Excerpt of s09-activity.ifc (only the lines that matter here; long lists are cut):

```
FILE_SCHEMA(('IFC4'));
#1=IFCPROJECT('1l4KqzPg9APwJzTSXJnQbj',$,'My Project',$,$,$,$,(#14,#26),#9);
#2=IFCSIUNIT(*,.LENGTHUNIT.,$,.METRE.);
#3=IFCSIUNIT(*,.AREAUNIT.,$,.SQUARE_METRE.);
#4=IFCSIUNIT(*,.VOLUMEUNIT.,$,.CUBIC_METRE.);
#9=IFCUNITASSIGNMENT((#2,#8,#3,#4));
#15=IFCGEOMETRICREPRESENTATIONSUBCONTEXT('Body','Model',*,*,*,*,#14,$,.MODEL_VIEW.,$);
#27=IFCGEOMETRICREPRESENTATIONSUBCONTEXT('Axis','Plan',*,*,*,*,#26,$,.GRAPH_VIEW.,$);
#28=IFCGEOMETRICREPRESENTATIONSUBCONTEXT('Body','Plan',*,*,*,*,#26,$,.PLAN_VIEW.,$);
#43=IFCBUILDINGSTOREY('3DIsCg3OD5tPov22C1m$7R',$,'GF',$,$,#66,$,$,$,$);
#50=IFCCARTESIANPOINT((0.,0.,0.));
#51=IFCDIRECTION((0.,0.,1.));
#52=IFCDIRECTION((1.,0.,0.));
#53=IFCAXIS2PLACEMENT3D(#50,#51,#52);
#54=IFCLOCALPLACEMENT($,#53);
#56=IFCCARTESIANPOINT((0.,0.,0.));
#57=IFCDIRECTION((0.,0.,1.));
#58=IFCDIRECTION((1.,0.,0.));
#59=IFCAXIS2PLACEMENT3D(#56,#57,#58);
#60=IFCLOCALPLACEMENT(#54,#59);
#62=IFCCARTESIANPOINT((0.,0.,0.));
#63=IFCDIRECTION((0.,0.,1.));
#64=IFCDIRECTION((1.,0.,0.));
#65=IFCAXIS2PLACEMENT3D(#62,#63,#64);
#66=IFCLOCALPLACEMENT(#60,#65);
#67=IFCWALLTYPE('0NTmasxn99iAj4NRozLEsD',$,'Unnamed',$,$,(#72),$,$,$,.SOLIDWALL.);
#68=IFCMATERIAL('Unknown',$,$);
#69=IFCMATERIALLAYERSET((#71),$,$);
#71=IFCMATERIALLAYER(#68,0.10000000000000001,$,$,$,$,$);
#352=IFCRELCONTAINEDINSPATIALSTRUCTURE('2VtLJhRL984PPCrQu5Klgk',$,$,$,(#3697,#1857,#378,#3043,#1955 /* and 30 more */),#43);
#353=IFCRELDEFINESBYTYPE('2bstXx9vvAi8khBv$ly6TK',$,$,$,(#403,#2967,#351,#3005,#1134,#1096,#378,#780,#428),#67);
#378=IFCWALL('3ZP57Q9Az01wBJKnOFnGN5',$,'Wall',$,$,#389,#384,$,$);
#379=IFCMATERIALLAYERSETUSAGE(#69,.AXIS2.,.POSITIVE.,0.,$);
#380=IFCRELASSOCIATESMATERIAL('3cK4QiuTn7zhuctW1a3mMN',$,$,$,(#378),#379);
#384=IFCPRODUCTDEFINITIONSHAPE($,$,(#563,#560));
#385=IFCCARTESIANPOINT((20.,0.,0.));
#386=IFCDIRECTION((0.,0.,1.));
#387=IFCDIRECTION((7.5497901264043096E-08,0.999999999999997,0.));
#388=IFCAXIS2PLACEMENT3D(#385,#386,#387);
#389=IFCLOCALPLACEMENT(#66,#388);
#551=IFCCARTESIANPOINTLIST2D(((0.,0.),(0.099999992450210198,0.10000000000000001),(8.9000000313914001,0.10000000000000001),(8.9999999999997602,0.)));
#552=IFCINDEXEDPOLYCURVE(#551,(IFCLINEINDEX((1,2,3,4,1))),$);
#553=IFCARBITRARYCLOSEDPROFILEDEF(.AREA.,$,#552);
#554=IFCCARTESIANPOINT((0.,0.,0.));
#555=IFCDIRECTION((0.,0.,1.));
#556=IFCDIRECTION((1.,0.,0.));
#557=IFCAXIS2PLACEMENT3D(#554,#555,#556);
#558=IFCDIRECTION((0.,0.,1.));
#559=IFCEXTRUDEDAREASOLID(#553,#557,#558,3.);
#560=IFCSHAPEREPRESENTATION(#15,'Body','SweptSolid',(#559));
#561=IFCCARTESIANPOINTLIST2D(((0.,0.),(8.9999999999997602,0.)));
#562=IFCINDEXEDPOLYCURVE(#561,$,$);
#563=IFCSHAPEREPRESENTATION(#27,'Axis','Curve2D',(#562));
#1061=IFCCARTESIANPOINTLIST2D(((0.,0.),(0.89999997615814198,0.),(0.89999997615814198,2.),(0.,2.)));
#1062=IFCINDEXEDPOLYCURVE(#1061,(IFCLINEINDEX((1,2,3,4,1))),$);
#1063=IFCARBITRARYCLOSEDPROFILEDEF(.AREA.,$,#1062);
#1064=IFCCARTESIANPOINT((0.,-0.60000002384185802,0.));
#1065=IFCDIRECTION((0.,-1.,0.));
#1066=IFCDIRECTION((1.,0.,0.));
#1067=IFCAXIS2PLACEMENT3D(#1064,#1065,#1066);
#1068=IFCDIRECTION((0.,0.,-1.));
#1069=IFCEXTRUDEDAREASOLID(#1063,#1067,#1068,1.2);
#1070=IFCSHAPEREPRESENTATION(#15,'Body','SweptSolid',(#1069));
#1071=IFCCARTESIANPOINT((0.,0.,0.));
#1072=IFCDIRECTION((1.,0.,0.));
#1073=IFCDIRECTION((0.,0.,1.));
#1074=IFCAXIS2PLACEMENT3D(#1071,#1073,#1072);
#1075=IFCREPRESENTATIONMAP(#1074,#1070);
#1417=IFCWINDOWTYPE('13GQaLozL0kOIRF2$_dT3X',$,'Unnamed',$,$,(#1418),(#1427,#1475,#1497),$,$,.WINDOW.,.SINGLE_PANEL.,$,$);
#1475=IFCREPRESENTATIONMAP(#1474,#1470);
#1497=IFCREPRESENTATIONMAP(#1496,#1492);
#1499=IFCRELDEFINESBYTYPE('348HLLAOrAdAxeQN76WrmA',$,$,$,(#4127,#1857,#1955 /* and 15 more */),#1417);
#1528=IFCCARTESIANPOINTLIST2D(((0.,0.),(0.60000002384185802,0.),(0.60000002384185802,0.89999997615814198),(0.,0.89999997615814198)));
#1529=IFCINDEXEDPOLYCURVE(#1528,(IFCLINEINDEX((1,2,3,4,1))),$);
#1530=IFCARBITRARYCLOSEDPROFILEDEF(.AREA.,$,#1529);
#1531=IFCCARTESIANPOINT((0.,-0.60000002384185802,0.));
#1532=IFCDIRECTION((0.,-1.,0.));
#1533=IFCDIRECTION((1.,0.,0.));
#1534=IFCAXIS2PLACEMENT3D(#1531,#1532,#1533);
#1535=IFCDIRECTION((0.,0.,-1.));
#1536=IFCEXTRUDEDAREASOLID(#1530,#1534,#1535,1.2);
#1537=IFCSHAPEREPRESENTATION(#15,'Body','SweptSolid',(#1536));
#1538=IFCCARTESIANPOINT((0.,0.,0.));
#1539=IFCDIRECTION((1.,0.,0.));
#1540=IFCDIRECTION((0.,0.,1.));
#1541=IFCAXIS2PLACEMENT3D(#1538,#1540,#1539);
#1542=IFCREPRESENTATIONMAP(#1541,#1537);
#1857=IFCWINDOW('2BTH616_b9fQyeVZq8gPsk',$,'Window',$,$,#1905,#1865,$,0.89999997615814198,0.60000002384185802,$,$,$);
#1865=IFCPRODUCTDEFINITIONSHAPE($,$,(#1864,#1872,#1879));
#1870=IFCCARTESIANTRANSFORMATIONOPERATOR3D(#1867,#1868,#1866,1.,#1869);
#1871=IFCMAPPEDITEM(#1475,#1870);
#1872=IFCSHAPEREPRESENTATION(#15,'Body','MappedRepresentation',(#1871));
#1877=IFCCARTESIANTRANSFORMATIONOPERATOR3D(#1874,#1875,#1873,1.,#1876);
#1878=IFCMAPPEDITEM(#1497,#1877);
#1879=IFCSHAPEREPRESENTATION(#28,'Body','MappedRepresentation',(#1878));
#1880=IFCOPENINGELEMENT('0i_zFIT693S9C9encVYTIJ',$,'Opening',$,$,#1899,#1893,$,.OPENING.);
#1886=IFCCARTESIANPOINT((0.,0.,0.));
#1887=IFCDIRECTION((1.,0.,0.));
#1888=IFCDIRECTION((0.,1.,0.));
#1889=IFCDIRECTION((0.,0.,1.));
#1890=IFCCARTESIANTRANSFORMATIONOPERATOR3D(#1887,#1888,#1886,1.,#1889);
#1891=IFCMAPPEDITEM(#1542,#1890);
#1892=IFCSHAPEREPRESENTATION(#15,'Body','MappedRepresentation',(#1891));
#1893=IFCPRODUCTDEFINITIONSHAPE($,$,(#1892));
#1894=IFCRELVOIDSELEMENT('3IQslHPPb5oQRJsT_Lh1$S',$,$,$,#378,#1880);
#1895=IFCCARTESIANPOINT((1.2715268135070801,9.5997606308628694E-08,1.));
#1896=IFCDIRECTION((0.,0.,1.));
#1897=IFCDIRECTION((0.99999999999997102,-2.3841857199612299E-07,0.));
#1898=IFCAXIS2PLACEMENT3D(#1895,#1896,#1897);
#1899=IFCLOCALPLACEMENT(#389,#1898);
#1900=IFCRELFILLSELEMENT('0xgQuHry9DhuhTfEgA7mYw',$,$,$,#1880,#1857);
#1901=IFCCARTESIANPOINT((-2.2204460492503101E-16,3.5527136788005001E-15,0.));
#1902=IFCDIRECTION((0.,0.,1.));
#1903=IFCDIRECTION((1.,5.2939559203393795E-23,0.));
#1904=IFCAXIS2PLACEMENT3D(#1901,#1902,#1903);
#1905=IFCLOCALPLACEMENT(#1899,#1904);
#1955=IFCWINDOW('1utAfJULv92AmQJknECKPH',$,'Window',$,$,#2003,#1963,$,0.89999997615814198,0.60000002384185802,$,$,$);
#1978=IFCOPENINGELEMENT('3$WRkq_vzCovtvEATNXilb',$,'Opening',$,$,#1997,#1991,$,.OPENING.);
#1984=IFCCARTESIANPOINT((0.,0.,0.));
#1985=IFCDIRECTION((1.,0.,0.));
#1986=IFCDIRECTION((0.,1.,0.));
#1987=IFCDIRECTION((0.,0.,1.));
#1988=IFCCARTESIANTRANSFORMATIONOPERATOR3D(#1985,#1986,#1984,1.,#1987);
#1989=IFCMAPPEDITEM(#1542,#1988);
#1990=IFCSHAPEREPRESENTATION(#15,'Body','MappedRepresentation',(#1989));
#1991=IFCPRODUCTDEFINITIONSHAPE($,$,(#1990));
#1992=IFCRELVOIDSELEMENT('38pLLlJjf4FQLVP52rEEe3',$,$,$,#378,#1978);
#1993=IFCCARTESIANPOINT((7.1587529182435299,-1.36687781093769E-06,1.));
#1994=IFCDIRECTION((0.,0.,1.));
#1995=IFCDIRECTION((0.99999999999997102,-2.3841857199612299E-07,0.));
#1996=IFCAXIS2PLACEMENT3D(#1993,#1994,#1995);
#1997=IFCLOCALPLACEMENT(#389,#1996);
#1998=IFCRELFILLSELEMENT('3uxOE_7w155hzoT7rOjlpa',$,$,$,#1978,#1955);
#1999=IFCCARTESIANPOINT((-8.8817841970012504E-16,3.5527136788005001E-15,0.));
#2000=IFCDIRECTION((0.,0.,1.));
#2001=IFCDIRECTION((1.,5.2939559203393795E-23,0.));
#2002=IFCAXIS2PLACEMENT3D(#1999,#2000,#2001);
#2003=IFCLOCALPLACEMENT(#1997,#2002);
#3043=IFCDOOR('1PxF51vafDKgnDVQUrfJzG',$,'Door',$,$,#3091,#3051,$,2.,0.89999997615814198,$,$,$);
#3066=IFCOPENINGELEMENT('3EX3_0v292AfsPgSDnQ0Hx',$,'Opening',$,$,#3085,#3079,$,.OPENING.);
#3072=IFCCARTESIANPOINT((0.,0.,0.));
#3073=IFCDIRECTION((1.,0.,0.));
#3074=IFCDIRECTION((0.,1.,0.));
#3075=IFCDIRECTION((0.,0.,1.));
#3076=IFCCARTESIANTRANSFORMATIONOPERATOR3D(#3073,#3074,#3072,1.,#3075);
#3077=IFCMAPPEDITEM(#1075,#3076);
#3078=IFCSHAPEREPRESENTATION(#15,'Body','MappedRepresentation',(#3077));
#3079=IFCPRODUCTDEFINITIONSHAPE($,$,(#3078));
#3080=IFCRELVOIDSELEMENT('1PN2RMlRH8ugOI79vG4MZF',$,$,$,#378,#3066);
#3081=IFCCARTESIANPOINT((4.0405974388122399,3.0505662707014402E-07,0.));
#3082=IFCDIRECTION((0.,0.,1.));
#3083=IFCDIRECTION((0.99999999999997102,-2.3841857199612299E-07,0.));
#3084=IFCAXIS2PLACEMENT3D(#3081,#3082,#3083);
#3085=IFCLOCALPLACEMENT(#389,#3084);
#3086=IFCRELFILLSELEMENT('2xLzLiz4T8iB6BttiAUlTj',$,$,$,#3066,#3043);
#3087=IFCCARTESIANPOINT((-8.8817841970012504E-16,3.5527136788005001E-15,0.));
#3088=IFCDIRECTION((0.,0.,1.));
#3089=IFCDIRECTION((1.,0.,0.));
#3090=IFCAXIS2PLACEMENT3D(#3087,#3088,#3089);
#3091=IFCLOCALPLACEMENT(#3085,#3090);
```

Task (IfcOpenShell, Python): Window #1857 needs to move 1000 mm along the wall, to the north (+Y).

```python
import ifcopenshell
import ifcopenshell.api.geometry
import ifcopenshell.util.placement

model = ifcopenshell.open("s09-activity.ifc")

window = model.by_guid("2BTH616_b9fQyeVZq8gPsk")
opening = window.FillsVoids[0].RelatingOpeningElement
wall = opening.VoidsElements[0].RelatingBuildingElement

wall_matrix = ifcopenshell.util.placement.get_local_placement(wall.ObjectPlacement)
shift = wall_matrix[:3, 0] * 1.0
before = ifcopenshell.util.placement.get_local_placement(window.ObjectPlacement)[:3, 3].copy()

# The window is placed relative to its opening, so it follows when the opening moves.
matrix = ifcopenshell.util.placement.get_local_placement(opening.ObjectPlacement)
matrix[:3, 3] += shift
ifcopenshell.api.geometry.edit_object_placement(
    model, product=opening, matrix=matrix, is_si=False, should_transform_children=True
)

after = ifcopenshell.util.placement.get_local_placement(window.ObjectPlacement)[:3, 3]
print("window moved by", (after - before).round(3) + 0.0)

model.write("s09-activity_updated.ifc")
```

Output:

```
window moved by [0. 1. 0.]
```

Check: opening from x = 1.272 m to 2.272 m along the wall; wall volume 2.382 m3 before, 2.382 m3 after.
